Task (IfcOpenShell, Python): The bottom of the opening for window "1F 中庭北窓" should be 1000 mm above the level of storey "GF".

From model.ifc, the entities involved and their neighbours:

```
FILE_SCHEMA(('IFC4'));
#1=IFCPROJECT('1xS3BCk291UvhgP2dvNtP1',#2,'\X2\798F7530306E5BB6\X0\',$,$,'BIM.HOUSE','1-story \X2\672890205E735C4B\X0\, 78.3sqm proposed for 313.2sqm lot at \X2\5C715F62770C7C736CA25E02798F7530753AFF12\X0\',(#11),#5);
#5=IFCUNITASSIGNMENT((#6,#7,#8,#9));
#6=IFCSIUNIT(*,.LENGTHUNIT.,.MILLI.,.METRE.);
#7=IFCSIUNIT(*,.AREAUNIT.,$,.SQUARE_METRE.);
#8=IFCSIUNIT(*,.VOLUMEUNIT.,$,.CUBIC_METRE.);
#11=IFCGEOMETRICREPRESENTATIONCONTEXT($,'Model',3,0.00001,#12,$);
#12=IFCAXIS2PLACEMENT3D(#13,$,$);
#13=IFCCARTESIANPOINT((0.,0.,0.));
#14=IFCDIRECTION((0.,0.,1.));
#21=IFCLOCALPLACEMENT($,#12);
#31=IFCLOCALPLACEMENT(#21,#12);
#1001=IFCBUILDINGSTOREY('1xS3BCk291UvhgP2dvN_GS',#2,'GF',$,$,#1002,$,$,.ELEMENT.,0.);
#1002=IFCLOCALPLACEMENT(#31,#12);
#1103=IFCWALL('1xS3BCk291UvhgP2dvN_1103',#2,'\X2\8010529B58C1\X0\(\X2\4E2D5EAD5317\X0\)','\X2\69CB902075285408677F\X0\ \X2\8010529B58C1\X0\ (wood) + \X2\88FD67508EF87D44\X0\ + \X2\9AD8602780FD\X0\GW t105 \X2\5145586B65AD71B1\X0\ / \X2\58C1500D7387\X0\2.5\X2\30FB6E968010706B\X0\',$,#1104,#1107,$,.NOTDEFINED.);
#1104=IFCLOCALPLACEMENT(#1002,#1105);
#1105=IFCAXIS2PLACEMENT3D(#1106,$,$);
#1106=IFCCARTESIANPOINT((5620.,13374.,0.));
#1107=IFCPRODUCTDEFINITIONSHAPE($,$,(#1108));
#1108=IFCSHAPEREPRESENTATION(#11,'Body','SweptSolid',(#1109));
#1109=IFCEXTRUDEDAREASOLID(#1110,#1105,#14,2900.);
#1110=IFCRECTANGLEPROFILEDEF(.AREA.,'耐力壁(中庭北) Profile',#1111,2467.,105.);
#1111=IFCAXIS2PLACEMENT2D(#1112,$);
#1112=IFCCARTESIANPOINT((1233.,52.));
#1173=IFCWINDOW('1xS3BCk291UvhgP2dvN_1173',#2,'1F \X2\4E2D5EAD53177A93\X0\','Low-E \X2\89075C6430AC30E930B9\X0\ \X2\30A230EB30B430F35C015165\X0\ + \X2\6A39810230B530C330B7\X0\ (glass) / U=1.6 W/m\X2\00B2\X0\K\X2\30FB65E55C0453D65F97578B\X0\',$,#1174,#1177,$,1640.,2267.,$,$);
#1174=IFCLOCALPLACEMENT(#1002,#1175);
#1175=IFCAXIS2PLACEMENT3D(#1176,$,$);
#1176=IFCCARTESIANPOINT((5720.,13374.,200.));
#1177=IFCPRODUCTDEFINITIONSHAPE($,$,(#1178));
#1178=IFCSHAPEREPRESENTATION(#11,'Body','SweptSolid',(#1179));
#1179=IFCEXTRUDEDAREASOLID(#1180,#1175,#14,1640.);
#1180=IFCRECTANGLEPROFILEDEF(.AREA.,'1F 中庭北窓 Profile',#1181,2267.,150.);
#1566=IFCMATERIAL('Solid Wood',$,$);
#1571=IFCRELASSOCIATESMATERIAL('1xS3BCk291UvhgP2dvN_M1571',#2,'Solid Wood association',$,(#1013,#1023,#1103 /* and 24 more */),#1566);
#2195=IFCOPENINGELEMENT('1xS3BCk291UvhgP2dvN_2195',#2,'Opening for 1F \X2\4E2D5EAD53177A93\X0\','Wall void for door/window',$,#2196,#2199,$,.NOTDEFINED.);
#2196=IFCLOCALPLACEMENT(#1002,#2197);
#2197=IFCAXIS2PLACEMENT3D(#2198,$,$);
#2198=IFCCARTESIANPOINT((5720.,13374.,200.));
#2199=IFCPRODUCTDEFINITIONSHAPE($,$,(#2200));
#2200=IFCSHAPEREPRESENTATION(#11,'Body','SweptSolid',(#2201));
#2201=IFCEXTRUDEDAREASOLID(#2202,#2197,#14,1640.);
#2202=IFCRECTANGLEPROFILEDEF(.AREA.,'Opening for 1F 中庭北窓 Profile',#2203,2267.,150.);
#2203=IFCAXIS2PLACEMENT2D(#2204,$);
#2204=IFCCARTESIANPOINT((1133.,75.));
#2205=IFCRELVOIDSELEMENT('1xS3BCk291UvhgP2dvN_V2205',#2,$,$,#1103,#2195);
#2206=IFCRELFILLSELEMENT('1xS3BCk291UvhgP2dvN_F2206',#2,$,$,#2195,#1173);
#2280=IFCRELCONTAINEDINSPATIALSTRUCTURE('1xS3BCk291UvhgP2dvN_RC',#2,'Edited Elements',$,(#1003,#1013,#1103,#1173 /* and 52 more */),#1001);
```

```python
import numpy as np
import ifcopenshell
import ifcopenshell.api.geometry
import ifcopenshell.geom
import ifcopenshell.util.element
import ifcopenshell.util.placement
import ifcopenshell.util.shape
import ifcopenshell.util.unit

model = ifcopenshell.open("model.ifc")
unit_scale = ifcopenshell.util.unit.calculate_unit_scale(model)

window = model.by_guid("1xS3BCk291UvhgP2dvN_1173")
opening = window.FillsVoids[0].RelatingOpeningElement
storey = ifcopenshell.util.element.get_container(window, ifc_class="IfcBuildingStorey")
level = ifcopenshell.util.placement.get_local_placement(storey.ObjectPlacement)[2, 3]

# The opening's origin need not be at the sill, so measure its lowest point.
shape = ifcopenshell.geom.create_shape(ifcopenshell.geom.settings(), opening)
bottom = ifcopenshell.util.shape.get_shape_bottom_elevation(shape, shape.geometry) / unit_scale
dz = level + 1000.0 - bottom

shift = np.array([0.0, 0.0, dz])
# The window is not placed relative to its opening, so move both.
for product in (opening, window):
    matrix = ifcopenshell.util.placement.get_local_placement(product.ObjectPlacement)
    matrix[:3, 3] += shift
    ifcopenshell.api.geometry.edit_object_placement(model, product=product, matrix=matrix, is_si=False)

print(f"moved by {dz * unit_scale:+.3f} m")

model.write("model_v2.ifc")
```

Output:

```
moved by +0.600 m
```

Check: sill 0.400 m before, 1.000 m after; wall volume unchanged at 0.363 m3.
